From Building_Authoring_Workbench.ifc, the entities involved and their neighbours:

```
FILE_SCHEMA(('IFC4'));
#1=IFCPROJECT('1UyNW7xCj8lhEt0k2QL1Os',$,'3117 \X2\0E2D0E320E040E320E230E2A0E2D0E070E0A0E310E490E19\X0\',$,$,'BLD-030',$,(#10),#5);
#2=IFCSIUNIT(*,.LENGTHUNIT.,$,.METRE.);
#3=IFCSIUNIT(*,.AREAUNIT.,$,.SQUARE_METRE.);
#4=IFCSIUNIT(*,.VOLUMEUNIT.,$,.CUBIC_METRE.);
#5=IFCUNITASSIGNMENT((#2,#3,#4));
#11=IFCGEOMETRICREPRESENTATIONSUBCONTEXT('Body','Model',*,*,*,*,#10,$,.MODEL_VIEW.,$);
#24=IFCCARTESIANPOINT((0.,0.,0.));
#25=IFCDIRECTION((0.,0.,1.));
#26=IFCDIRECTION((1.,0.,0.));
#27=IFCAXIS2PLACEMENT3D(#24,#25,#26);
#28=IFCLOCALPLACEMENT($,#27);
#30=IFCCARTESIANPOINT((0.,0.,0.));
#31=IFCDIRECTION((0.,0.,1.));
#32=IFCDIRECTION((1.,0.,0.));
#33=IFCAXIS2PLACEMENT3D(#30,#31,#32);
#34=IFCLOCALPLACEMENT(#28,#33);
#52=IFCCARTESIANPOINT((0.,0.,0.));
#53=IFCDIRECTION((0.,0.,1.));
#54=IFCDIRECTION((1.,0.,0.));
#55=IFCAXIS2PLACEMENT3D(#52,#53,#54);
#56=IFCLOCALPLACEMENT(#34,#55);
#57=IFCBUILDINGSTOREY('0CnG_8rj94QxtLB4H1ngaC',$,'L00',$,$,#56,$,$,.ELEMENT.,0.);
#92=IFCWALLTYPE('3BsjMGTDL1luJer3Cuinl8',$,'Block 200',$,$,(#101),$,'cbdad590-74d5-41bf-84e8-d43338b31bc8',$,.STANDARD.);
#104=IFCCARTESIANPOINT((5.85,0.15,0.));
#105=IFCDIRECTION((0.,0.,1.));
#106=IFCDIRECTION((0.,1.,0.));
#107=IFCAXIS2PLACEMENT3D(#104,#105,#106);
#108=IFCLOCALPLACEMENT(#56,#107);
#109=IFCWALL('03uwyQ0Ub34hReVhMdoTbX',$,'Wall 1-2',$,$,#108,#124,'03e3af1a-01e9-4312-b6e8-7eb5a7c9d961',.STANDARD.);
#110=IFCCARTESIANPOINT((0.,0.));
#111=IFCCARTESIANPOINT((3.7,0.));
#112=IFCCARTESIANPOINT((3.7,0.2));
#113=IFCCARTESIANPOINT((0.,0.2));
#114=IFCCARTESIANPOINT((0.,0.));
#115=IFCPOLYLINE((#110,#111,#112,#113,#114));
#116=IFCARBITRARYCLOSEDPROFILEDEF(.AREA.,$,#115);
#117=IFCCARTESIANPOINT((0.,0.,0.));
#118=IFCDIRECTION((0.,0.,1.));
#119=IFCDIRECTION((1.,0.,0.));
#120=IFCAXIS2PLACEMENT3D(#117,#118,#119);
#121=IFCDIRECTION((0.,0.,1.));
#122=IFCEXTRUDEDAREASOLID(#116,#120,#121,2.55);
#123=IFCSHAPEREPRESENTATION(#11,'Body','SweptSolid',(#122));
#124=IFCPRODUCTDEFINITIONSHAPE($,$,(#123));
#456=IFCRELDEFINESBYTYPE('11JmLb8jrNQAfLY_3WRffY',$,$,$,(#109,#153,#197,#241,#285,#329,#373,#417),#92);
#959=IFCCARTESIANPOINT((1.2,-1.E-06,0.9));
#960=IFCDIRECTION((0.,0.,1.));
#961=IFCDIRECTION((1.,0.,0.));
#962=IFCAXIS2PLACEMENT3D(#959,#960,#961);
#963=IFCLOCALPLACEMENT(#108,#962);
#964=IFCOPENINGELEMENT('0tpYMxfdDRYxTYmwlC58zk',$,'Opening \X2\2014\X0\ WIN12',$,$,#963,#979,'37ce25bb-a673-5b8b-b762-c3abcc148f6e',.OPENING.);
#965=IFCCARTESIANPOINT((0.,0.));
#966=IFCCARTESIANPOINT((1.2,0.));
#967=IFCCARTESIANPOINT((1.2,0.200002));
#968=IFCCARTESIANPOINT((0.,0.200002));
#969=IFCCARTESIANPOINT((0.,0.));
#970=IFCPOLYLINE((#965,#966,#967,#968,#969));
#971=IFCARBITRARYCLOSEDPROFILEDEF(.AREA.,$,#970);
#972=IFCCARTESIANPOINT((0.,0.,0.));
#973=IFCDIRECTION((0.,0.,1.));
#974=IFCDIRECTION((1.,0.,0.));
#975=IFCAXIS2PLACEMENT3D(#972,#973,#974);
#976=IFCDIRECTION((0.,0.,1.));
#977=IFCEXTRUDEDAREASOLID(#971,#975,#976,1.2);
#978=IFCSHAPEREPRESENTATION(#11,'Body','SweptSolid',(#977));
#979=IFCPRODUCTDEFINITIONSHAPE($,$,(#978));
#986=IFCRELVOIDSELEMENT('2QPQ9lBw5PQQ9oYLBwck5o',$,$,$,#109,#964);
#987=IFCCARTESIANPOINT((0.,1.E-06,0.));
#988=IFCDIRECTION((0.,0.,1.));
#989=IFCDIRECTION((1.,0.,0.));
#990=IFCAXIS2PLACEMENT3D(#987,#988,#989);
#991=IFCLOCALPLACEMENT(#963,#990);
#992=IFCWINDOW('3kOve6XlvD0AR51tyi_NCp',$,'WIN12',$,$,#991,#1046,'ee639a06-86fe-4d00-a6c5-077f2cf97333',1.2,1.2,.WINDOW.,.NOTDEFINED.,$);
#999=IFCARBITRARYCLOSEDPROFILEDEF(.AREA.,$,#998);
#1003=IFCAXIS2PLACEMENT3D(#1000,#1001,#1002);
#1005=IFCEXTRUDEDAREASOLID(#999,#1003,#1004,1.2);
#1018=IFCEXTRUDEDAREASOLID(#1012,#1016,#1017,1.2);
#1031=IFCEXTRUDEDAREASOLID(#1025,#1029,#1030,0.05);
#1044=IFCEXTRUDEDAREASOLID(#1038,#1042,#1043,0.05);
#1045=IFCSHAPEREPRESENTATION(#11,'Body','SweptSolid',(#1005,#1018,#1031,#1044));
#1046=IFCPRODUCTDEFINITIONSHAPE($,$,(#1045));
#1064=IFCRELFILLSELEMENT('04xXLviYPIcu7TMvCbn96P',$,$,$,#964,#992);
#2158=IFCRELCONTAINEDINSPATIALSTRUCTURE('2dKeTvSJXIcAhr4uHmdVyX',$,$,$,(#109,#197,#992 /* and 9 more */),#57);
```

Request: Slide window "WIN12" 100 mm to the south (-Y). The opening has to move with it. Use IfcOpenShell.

```python
import ifcopenshell
import ifcopenshell.api.geometry
import ifcopenshell.util.placement
import ifcopenshell.util.unit

model = ifcopenshell.open("Building_Authoring_Workbench.ifc")
unit_scale = ifcopenshell.util.unit.calculate_unit_scale(model)

window = model.by_guid("3kOve6XlvD0AR51tyi_NCp")
opening = window.FillsVoids[0].RelatingOpeningElement
wall = opening.VoidsElements[0].RelatingBuildingElement

wall_matrix = ifcopenshell.util.placement.get_local_placement(wall.ObjectPlacement)
shift = wall_matrix[:3, 0] * -0.1 / unit_scale
before = ifcopenshell.util.placement.get_local_placement(window.ObjectPlacement)[:3, 3].copy()

# The window is placed relative to its opening, so it follows when the opening moves.
matrix = ifcopenshell.util.placement.get_local_placement(opening.ObjectPlacement)
matrix[:3, 3] += shift
ifcopenshell.api.geometry.edit_object_placement(
    model, product=opening, matrix=matrix, is_si=False, should_transform_children=True
)

after = ifcopenshell.util.placement.get_local_placement(window.ObjectPlacement)[:3, 3]
print("window moved by", (after - before).round(3) + 0.0)

model.write("Building_Authoring_Workbench-out.ifc")
```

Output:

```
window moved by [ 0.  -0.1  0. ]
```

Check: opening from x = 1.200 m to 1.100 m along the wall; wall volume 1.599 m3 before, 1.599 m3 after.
